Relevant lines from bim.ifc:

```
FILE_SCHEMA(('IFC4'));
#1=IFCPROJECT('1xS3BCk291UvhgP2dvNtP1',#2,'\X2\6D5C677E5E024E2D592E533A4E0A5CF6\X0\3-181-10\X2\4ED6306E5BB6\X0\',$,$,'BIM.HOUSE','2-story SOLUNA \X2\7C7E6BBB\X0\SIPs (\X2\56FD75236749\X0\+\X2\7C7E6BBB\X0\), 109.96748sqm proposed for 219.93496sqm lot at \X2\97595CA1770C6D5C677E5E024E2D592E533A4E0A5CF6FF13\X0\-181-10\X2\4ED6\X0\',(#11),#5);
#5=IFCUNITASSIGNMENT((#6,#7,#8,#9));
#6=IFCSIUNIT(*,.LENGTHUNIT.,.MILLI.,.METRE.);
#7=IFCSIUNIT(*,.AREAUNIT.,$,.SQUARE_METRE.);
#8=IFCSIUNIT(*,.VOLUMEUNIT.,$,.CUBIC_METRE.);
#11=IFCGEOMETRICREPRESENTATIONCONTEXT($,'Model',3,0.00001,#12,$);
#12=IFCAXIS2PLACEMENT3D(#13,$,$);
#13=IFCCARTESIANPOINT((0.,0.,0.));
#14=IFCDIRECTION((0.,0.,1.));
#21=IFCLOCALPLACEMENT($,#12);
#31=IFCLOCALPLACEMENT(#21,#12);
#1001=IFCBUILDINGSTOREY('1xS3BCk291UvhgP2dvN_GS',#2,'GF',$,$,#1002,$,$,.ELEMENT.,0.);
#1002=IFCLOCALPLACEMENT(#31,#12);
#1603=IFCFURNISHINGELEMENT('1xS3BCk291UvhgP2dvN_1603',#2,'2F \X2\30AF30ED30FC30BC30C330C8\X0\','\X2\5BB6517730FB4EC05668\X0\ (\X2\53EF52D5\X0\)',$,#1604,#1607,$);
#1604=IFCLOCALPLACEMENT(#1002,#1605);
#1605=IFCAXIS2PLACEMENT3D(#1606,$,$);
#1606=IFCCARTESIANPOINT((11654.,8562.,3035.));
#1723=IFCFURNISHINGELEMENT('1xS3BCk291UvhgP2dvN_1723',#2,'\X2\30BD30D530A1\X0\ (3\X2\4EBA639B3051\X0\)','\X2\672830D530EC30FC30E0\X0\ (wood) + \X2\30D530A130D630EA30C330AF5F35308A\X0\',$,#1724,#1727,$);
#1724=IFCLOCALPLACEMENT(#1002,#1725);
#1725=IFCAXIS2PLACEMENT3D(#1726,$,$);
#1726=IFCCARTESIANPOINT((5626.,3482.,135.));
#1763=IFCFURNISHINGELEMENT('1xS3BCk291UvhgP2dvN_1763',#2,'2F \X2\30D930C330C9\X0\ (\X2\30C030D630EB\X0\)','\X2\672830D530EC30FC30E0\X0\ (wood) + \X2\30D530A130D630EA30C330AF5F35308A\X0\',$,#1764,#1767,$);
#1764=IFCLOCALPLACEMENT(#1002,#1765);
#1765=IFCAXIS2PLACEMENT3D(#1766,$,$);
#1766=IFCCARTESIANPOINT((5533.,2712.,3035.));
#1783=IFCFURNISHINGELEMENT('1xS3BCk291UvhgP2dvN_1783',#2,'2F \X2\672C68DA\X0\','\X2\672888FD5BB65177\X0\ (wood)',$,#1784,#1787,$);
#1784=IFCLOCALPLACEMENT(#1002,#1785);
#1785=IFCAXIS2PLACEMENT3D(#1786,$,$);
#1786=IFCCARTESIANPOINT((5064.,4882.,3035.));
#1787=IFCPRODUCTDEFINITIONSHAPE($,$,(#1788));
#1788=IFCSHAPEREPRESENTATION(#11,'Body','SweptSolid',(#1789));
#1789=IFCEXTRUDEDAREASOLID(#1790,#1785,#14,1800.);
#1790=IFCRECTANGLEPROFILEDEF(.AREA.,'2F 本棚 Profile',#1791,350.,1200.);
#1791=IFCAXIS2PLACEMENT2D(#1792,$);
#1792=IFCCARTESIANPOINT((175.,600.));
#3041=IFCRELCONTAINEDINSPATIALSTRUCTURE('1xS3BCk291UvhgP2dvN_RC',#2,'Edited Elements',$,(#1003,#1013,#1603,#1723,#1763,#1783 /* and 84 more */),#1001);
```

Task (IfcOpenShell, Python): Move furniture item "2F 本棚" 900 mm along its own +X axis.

```python
import ifcopenshell
import ifcopenshell.api.geometry
import ifcopenshell.util.placement
import ifcopenshell.util.unit

model = ifcopenshell.open("bim.ifc")
unit_scale = ifcopenshell.util.unit.calculate_unit_scale(model)

item = model.by_guid("1xS3BCk291UvhgP2dvN_1783")
matrix = ifcopenshell.util.placement.get_local_placement(item.ObjectPlacement)
matrix[:3, 3] += matrix[:3, 0] * 0.9 / unit_scale
ifcopenshell.api.geometry.edit_object_placement(model, product=item, matrix=matrix, is_si=False)

print(ifcopenshell.util.placement.get_local_placement(item.ObjectPlacement).round(3) + 0.0)

model.write("bim_rev.ifc")
```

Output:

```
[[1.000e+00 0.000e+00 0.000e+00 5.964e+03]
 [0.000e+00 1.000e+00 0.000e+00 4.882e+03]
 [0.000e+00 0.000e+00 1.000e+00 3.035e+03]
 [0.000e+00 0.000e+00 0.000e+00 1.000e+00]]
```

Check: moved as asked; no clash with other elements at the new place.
